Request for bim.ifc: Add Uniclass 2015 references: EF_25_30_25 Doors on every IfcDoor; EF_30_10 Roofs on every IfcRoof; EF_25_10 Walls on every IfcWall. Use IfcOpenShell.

First a look at what the model holds.

```python
import ifcopenshell

model = ifcopenshell.open("bim.ifc")
print(model.schema)
print("classifications:", [c.Name for c in model.by_type("IfcClassification")])
for ifc_class in ("IfcDoor", "IfcRoof", "IfcStair", "IfcWall", "IfcWindow"):
    print(ifc_class, len(model.by_type(ifc_class)))
```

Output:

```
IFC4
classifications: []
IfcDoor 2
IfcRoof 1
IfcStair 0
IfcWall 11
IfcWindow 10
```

```python
import ifcopenshell
import ifcopenshell.api.classification

model = ifcopenshell.open("bim.ifc")

system = ifcopenshell.api.classification.add_classification(model, classification="Uniclass 2015")

codes = {
    "IfcDoor": ("EF_25_30_25", "Doors"),
    "IfcRoof": ("EF_30_10", "Roofs"),
    "IfcWall": ("EF_25_10", "Walls"),
}
for ifc_class, (code, name) in codes.items():
    products = model.by_type(ifc_class)
    ifcopenshell.api.classification.add_reference(
        model, products=products, classification=system, identification=code, name=name
    )
    print(code, len(products))

model.write("bim_edited.ifc")
```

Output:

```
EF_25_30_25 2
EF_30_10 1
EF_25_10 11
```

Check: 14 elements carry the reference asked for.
